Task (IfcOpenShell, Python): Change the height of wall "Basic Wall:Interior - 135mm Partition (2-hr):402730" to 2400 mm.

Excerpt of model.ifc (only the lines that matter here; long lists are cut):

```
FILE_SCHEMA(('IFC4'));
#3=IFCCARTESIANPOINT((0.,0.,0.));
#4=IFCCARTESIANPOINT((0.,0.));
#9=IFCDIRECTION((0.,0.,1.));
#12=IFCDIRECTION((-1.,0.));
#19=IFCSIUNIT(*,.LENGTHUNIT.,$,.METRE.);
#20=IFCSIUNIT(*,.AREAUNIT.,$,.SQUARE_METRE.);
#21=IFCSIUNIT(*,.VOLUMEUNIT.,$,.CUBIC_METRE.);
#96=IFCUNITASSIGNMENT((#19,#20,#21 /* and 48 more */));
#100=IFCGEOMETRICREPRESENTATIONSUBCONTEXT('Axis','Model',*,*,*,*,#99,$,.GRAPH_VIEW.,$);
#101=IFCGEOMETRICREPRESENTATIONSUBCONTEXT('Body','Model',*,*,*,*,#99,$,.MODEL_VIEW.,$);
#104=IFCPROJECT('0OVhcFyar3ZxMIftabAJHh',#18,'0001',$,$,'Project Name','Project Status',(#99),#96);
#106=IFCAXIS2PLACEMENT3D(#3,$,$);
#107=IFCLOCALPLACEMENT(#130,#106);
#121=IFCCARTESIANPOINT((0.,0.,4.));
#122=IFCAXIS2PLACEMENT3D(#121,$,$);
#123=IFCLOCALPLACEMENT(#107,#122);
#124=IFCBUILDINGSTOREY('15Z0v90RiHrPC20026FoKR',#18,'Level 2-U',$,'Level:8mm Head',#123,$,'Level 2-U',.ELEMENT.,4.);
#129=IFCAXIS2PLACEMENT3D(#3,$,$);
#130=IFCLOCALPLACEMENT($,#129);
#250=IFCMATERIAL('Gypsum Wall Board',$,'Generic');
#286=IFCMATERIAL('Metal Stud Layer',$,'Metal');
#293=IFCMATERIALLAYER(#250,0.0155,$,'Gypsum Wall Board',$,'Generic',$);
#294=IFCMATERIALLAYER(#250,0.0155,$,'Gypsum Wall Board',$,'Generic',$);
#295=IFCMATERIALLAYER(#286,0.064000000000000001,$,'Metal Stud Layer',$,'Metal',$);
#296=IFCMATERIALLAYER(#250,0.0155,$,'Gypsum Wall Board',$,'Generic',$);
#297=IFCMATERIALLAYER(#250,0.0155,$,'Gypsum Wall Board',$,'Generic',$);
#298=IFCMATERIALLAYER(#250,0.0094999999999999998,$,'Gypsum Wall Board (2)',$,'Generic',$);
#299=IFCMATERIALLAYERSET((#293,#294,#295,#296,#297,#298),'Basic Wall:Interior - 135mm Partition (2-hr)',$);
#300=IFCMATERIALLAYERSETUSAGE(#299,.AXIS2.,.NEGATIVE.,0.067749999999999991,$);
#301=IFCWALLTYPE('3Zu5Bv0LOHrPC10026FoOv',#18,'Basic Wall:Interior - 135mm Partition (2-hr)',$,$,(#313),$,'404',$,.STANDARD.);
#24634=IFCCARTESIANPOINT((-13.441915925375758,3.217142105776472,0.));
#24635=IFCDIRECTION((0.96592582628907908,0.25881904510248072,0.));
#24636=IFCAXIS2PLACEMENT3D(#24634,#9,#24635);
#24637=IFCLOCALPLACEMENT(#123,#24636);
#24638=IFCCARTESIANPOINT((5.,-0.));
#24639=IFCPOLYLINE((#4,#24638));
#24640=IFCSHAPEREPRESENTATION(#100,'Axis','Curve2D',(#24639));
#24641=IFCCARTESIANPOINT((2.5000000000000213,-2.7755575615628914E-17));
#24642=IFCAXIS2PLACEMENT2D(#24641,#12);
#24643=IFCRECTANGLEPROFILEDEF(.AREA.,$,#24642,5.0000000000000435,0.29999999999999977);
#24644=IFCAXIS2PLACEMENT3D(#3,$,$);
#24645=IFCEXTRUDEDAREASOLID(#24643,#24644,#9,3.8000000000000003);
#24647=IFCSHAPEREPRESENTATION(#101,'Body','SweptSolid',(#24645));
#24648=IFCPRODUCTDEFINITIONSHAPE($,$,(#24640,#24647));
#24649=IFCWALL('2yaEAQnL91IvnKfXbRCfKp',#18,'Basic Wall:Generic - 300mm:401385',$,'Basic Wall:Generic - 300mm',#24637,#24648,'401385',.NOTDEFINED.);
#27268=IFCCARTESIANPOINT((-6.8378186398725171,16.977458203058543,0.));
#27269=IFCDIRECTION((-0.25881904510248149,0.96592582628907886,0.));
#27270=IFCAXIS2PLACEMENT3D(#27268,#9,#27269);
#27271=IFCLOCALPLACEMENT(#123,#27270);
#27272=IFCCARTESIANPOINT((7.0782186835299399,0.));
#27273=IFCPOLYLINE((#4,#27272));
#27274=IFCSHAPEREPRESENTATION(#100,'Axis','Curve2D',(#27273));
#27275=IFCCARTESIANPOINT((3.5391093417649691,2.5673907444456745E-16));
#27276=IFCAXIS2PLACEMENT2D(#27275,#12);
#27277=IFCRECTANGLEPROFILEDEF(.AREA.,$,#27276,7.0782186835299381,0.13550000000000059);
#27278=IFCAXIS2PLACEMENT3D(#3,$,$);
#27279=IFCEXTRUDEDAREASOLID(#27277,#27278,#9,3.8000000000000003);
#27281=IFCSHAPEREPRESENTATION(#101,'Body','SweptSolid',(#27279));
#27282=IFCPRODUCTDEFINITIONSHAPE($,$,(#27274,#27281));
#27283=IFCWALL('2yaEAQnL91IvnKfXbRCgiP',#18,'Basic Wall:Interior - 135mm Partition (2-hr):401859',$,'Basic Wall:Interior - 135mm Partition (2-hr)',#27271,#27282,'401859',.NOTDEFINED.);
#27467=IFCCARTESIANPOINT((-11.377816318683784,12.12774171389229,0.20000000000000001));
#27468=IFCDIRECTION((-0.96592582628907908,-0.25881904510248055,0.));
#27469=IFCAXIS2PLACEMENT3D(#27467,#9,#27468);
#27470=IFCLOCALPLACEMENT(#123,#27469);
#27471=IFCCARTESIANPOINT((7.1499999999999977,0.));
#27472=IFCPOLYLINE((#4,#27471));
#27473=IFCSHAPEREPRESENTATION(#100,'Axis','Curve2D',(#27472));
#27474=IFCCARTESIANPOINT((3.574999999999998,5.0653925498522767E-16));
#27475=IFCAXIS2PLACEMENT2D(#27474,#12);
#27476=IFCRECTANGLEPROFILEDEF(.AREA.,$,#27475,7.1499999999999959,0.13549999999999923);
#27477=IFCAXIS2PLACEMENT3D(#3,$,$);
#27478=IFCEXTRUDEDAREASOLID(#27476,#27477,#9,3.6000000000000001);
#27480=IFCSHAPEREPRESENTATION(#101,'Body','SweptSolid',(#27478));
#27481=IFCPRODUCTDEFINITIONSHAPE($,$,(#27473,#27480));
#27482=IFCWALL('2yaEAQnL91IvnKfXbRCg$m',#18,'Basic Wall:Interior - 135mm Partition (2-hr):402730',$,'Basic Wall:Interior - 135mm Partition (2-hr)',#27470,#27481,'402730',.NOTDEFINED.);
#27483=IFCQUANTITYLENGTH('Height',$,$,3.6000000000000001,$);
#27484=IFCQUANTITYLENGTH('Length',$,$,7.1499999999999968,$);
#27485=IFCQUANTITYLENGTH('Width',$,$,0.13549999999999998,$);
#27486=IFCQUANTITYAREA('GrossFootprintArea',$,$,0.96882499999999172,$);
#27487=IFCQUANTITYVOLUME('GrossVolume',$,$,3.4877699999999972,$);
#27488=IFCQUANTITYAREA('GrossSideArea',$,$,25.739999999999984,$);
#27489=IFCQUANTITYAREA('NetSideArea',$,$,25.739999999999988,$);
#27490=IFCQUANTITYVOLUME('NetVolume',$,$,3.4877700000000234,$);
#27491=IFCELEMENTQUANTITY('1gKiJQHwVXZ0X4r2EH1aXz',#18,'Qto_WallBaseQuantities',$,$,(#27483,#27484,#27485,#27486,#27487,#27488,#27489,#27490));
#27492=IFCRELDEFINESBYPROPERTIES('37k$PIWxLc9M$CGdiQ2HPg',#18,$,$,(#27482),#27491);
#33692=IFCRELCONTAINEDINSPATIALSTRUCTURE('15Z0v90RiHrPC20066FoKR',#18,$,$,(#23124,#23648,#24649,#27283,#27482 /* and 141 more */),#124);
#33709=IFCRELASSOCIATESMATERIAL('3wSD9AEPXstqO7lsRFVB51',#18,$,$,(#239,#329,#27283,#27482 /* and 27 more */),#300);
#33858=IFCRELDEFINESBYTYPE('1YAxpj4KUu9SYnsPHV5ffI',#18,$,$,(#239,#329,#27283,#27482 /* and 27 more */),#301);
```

```python
import ifcopenshell
import ifcopenshell.api.pset
import ifcopenshell.geom
import ifcopenshell.util.element
import ifcopenshell.util.representation
import ifcopenshell.util.shape
import ifcopenshell.util.unit

model = ifcopenshell.open("model.ifc")
unit_scale = ifcopenshell.util.unit.calculate_unit_scale(model)
area_scale = ifcopenshell.util.unit.calculate_unit_scale(model, "AREAUNIT")
volume_scale = ifcopenshell.util.unit.calculate_unit_scale(model, "VOLUMEUNIT")
settings = ifcopenshell.geom.settings()


def volume(element):
    """Net volume in cubic metres, openings subtracted."""
    shape = ifcopenshell.geom.create_shape(settings, element)
    return ifcopenshell.util.shape.get_volume(shape.geometry)


wall = model.by_id(27482)
before = volume(wall)

body = ifcopenshell.util.representation.get_representation(wall, "Model", "Body")
solid = body.Items[0]
old_height = solid.Depth
solid.Depth = 2.4
after = volume(wall)
thickness = 0.1355  # wall thickness in metres

# Update the stored height, areas and volumes.
qto = model.by_id(ifcopenshell.util.element.get_pset(wall, "Qto_WallBaseQuantities", should_inherit=False)["id"])
ifcopenshell.api.pset.edit_qto(model, qto=qto, properties={
    "Height": solid.Depth,
    "GrossVolume": ifcopenshell.util.element.get_pset(wall, "Qto_WallBaseQuantities", "GrossVolume") * solid.Depth / old_height,
    "GrossSideArea": ifcopenshell.util.element.get_pset(wall, "Qto_WallBaseQuantities", "GrossSideArea") * solid.Depth / old_height,
    "NetSideArea": after / thickness / area_scale,
    "NetVolume": after / volume_scale,
})

print(f"height {old_height:g} -> {solid.Depth:g}, volume {before:.3f} -> {after:.3f} m3")

model.write("model_edited.ifc")
```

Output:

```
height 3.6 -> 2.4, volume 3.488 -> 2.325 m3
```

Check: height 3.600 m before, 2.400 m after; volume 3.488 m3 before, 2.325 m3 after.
